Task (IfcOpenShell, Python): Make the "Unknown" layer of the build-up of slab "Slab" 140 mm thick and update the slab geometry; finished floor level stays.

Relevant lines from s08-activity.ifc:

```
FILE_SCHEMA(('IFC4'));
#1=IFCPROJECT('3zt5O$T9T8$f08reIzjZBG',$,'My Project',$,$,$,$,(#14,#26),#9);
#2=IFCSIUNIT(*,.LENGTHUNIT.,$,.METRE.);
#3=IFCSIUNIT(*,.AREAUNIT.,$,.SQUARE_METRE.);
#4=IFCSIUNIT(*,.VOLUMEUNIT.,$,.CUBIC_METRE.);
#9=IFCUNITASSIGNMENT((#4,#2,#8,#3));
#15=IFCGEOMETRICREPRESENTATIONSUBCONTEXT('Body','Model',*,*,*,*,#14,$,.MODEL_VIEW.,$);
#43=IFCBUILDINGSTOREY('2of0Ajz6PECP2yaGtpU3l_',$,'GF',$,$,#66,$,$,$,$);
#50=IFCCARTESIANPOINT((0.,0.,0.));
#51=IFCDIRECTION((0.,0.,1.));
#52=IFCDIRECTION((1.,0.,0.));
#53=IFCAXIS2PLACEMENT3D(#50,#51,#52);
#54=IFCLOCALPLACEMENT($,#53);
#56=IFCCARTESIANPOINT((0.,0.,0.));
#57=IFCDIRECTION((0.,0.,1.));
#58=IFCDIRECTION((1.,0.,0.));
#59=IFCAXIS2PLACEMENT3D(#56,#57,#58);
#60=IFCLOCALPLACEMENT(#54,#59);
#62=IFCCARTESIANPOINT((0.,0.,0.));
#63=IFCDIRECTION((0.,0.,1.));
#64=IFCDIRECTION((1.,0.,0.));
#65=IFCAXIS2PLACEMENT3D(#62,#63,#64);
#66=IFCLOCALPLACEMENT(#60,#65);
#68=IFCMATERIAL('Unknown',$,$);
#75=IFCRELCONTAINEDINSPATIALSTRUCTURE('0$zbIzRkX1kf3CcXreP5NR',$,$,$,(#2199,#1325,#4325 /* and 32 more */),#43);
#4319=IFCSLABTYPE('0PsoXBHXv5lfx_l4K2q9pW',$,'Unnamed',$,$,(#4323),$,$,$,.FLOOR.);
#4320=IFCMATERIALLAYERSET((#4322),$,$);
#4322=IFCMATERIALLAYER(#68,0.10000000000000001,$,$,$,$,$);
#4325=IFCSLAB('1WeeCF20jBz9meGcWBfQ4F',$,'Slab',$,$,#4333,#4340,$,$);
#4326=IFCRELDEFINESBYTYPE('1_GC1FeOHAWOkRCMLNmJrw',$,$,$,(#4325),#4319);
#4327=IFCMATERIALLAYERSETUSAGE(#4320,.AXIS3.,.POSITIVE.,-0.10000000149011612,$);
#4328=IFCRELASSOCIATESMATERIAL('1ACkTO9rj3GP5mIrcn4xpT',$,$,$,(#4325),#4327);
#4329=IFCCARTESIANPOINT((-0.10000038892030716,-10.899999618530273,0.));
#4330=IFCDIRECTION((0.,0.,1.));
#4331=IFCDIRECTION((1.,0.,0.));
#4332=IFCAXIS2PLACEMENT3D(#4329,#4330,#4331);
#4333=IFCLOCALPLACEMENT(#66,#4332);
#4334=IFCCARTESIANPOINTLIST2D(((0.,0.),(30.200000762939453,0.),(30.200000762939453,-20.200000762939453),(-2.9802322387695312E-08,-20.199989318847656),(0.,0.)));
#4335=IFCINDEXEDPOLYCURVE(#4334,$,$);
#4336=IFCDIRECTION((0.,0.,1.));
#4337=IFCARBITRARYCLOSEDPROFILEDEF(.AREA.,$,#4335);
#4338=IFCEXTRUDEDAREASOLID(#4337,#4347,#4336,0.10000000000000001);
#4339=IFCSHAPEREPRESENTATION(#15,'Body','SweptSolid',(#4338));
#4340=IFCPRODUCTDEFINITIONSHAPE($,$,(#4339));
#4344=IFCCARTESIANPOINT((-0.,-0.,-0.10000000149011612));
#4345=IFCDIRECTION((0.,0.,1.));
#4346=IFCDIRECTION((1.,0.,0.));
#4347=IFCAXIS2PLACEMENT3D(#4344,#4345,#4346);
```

```python
import ifcopenshell
import ifcopenshell.util.element
import ifcopenshell.util.representation

model = ifcopenshell.open("s08-activity.ifc")

layer_set = model.by_id(4320)
layer = next(l for l in layer_set.MaterialLayers if l.Material and l.Material.Name == "Unknown")
change = 0.14 - layer.LayerThickness
layer.LayerThickness += change

# Geometry does not follow the layer set by itself.
slabs = [e for e in ifcopenshell.util.element.get_elements_by_material(model, layer_set) if e.is_a("IfcSlab")]
for slab in sorted(slabs, key=lambda e: e.id()):
    body = ifcopenshell.util.representation.get_representation(slab, "Model", "Body")
    solid = body.Items[0]
    old_depth = solid.Depth
    solid.Depth += change
    # Extruded upwards: lower the start of the extrusion so the top stays.
    x, y, z = solid.Position.Location.Coordinates
    solid.Position.Location = model.createIfcCartesianPoint((x, y, z - change))
    print(slab.id(), f"{old_depth:g} -> {solid.Depth:g}")

# The layers are counted up from the underside, which has moved.
for usage in {ifcopenshell.util.element.get_material(slab) for slab in slabs}:
    usage.OffsetFromReferenceLine -= change

model.write("s08-activity_v2.ifc")
```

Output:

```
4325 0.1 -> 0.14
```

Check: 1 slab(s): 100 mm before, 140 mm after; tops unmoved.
